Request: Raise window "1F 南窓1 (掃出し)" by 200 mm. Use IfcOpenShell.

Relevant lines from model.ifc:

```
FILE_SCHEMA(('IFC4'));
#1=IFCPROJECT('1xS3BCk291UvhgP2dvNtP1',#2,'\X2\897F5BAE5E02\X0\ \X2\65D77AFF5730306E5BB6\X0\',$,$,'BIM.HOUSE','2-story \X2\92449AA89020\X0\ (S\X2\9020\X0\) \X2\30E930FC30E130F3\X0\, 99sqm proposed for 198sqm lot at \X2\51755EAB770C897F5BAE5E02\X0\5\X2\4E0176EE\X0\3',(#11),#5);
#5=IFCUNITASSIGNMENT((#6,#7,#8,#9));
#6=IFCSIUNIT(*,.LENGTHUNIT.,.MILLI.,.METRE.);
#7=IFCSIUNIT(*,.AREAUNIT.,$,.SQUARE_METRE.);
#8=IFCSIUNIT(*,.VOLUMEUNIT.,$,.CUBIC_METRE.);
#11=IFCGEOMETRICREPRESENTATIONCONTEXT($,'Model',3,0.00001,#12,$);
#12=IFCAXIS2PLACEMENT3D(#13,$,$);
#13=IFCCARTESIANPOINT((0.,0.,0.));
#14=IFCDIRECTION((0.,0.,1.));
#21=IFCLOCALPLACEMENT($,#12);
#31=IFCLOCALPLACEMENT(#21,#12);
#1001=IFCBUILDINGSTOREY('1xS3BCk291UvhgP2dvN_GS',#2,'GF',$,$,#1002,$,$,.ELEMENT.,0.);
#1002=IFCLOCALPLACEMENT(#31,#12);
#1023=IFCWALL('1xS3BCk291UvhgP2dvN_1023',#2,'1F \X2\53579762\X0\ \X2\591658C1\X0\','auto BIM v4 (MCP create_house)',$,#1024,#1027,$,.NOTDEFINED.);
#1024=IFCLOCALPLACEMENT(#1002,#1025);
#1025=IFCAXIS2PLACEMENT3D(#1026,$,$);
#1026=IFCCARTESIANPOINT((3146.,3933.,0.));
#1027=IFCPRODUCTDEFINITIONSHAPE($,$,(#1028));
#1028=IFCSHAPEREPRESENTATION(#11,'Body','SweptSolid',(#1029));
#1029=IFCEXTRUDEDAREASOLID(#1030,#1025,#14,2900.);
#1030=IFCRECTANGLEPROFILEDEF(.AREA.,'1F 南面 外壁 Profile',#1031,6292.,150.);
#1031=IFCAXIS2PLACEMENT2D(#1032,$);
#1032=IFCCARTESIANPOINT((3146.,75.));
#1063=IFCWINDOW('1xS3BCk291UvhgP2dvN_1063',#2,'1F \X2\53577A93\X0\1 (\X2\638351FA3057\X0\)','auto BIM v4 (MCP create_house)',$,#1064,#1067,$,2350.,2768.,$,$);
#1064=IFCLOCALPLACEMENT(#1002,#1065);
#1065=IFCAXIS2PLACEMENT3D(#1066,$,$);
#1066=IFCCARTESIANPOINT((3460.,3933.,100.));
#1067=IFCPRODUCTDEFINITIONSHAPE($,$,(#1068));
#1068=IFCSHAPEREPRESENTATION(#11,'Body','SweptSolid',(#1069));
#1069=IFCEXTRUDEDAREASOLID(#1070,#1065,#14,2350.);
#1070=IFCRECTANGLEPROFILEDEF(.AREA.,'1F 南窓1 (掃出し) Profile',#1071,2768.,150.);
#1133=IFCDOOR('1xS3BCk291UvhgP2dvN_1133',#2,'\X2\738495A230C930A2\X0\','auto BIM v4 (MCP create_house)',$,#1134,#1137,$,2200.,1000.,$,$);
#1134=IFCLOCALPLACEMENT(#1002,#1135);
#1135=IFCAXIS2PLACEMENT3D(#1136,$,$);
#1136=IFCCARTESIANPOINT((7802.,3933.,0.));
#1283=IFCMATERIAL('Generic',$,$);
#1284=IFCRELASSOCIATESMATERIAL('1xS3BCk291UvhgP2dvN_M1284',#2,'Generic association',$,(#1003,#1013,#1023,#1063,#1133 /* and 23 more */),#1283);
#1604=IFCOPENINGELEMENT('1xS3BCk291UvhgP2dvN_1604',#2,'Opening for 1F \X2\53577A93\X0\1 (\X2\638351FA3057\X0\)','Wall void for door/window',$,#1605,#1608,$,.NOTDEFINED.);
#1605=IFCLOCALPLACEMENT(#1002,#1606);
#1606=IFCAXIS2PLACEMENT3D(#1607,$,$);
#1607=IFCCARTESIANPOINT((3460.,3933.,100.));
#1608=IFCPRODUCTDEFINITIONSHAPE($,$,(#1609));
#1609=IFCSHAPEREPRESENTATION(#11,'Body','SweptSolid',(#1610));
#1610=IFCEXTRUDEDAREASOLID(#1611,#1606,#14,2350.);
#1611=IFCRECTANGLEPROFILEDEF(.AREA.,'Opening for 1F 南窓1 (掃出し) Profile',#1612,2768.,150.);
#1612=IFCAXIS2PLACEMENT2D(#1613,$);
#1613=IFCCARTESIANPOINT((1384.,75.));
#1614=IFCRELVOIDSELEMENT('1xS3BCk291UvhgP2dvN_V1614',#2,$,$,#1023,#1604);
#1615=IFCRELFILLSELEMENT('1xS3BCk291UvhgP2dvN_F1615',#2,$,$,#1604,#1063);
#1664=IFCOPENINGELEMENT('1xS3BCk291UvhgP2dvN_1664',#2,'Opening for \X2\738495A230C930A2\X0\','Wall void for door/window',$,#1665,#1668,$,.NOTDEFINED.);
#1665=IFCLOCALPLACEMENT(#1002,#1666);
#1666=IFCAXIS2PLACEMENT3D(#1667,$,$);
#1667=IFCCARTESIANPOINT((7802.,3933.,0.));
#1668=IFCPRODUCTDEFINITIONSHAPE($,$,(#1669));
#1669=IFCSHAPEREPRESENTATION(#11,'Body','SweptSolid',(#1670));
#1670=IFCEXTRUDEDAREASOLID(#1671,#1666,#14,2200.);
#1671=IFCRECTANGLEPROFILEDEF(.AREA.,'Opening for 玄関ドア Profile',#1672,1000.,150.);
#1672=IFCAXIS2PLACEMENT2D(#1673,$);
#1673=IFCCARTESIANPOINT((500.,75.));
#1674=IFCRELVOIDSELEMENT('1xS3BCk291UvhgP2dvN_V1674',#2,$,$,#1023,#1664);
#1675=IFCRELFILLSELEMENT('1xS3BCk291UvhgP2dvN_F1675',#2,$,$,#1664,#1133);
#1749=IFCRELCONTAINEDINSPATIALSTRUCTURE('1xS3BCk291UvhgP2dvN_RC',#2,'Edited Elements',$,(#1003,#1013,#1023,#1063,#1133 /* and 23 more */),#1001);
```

```python
import numpy as np
import ifcopenshell
import ifcopenshell.api.geometry
import ifcopenshell.util.placement
import ifcopenshell.util.unit

model = ifcopenshell.open("model.ifc")
unit_scale = ifcopenshell.util.unit.calculate_unit_scale(model)

window = model.by_guid("1xS3BCk291UvhgP2dvN_1063")
opening = window.FillsVoids[0].RelatingOpeningElement
dz = 200.0

shift = np.array([0.0, 0.0, dz])
# The window is not placed relative to its opening, so move both.
for product in (opening, window):
    matrix = ifcopenshell.util.placement.get_local_placement(product.ObjectPlacement)
    matrix[:3, 3] += shift
    ifcopenshell.api.geometry.edit_object_placement(model, product=product, matrix=matrix, is_si=False)

print(f"moved by {dz * unit_scale:+.3f} m")

model.write("model_v2.ifc")
```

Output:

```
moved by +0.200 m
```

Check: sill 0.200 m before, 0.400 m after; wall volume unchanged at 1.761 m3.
